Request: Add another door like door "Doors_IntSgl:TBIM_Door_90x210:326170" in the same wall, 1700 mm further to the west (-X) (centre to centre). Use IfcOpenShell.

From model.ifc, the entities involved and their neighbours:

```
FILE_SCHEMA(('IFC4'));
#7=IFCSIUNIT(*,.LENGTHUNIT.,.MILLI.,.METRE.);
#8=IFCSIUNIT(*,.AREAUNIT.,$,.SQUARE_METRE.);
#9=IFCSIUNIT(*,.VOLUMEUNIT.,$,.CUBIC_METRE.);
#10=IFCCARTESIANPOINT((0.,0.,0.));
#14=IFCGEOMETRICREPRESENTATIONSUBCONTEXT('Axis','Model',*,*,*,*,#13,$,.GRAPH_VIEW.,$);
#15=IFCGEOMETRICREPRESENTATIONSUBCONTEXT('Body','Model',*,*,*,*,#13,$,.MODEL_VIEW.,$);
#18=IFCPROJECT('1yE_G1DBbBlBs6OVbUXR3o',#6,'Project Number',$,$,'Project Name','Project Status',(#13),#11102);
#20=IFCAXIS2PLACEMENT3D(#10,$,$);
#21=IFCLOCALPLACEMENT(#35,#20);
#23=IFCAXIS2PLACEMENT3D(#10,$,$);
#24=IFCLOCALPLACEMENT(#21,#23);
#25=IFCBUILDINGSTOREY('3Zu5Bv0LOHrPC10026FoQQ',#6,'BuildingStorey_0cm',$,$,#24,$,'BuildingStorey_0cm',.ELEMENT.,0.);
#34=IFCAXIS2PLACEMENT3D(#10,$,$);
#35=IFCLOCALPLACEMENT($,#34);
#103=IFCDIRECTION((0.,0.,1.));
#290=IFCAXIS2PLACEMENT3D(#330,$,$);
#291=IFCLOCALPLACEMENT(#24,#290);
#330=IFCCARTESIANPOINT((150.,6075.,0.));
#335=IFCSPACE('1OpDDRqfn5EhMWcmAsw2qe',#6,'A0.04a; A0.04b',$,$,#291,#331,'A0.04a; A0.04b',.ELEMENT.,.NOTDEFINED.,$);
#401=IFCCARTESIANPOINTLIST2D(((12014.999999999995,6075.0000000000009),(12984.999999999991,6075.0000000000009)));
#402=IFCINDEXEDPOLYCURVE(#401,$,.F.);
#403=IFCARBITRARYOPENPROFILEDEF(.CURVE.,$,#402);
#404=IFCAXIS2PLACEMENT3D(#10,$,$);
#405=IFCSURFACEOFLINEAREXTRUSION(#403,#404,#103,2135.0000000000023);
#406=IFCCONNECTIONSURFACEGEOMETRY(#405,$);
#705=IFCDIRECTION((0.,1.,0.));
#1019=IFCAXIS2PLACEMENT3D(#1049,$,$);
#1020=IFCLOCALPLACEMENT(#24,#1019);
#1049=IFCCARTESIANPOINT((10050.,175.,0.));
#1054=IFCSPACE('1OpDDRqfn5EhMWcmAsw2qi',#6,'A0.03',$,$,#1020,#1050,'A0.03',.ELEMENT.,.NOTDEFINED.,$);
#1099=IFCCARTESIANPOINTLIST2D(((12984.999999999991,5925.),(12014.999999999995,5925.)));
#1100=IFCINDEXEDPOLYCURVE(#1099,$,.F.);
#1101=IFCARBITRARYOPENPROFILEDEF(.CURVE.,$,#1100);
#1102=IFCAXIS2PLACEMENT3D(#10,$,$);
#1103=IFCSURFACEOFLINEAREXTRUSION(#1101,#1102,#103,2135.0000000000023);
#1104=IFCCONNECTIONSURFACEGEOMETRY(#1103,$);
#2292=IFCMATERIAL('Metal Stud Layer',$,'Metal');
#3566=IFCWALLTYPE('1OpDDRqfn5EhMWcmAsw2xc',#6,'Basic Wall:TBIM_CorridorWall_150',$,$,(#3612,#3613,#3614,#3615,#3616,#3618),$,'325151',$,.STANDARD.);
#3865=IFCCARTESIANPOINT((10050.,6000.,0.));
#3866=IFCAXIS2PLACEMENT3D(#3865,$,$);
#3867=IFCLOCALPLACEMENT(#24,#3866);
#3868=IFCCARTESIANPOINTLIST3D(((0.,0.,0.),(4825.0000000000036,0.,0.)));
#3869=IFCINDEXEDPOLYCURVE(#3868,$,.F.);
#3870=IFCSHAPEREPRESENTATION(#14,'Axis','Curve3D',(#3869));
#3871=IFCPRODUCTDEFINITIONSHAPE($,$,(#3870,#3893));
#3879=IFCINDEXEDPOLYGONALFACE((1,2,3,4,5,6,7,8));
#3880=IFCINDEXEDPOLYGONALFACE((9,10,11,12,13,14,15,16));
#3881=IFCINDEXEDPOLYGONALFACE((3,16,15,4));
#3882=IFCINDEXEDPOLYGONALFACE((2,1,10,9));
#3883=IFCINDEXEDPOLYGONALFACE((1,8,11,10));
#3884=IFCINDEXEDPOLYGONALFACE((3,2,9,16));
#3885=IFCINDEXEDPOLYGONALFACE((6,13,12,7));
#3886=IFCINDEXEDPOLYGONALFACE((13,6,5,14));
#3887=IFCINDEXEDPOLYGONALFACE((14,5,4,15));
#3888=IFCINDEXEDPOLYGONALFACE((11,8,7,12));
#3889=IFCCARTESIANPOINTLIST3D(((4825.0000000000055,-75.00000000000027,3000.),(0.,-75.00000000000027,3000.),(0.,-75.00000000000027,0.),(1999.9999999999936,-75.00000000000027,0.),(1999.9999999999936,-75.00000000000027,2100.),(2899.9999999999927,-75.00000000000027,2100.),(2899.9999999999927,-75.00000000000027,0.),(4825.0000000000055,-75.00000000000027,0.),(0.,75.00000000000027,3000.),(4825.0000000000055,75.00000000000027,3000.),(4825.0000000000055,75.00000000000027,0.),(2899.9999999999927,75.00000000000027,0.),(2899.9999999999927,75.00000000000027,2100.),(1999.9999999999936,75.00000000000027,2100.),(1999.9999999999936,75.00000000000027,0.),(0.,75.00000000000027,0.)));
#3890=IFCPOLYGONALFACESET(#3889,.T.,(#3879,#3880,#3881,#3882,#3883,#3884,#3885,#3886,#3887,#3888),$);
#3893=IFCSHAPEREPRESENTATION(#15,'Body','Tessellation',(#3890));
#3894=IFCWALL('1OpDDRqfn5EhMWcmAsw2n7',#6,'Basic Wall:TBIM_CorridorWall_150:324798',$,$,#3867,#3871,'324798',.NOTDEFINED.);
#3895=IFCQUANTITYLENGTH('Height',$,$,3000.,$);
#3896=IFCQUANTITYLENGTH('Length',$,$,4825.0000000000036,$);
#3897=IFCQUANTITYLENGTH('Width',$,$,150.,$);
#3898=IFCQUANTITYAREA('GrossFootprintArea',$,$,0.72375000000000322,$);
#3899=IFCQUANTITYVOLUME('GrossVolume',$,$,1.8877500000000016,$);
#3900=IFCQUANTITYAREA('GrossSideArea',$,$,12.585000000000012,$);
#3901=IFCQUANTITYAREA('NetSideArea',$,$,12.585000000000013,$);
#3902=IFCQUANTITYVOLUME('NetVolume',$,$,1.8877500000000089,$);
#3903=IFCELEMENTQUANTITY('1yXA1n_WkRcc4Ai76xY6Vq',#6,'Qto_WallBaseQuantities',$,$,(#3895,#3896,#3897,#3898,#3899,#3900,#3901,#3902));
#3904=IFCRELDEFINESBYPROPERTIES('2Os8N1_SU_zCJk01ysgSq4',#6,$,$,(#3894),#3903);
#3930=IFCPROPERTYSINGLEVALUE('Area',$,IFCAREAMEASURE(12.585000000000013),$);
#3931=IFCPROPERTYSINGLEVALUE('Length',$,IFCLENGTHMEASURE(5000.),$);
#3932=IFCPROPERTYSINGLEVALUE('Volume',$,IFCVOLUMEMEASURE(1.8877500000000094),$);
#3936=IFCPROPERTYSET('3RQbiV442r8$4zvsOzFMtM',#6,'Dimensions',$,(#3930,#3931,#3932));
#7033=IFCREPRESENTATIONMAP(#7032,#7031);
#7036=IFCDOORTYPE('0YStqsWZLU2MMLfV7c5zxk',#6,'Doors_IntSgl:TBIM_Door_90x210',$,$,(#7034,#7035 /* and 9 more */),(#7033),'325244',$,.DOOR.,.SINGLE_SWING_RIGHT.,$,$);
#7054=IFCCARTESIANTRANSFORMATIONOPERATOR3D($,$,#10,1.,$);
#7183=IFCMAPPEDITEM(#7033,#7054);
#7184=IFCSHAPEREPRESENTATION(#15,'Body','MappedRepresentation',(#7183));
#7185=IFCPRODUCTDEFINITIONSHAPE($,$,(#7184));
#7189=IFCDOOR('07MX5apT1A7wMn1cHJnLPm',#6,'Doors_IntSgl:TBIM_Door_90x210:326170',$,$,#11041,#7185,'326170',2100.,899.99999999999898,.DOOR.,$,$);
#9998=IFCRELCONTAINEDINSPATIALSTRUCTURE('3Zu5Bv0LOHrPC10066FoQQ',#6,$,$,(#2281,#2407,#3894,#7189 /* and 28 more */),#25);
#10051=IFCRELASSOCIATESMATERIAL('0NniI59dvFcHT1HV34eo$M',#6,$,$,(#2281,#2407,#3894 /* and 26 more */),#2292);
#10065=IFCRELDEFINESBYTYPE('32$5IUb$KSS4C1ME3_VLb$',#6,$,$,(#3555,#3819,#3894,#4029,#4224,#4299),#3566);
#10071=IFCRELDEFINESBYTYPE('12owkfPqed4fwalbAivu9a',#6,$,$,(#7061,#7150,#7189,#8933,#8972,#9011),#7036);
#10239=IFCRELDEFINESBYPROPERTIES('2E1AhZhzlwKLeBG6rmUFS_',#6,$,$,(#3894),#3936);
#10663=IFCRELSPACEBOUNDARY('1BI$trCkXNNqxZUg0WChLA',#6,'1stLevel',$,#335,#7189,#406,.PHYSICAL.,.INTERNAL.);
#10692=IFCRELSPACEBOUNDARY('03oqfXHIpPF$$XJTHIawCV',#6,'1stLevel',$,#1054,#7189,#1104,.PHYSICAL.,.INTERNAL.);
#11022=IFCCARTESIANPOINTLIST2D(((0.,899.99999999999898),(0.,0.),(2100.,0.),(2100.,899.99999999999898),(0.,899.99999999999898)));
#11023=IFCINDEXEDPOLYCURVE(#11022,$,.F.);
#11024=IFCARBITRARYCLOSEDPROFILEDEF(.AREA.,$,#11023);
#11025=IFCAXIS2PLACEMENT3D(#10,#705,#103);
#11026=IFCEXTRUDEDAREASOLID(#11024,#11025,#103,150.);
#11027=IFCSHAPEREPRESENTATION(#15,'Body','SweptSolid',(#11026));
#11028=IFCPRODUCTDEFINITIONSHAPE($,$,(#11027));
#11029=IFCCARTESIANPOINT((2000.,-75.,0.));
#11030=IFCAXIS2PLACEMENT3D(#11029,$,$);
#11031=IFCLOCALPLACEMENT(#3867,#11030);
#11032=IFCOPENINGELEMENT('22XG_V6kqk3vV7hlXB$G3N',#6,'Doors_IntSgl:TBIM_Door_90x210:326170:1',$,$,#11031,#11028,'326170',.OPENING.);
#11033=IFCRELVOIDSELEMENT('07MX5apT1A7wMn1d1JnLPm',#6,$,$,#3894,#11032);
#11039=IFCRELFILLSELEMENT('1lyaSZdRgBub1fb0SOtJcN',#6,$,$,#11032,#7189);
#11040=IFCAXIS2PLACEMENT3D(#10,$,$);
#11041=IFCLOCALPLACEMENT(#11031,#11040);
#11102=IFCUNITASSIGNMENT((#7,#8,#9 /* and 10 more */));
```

```python
import numpy as np
import ifcopenshell
import ifcopenshell.api.feature
import ifcopenshell.api.geometry
import ifcopenshell.api.pset
import ifcopenshell.api.root
import ifcopenshell.geom
import ifcopenshell.util.element
import ifcopenshell.util.placement
import ifcopenshell.util.shape
import ifcopenshell.util.unit

model = ifcopenshell.open("model.ifc")
unit_scale = ifcopenshell.util.unit.calculate_unit_scale(model)
area_scale = ifcopenshell.util.unit.calculate_unit_scale(model, "AREAUNIT")
volume_scale = ifcopenshell.util.unit.calculate_unit_scale(model, "VOLUMEUNIT")
settings = ifcopenshell.geom.settings()


def volume(element):
    """Net volume in cubic metres, openings subtracted."""
    shape = ifcopenshell.geom.create_shape(settings, element)
    return ifcopenshell.util.shape.get_volume(shape.geometry)


def reuse_history(source, copy):
    """copy_class also copies each property set's owner history, people and application; keep the originals."""
    for rel in copy.IsDefinedBy:
        if rel.is_a("IfcRelDefinesByProperties") and (history := rel.RelatingPropertyDefinition.OwnerHistory):
            rel.RelatingPropertyDefinition.OwnerHistory = source.OwnerHistory
            ifcopenshell.util.element.remove_deep2(model, history)


door = model.by_guid("07MX5apT1A7wMn1cHJnLPm")
opening = door.FillsVoids[0].RelatingOpeningElement
wall = opening.VoidsElements[0].RelatingBuildingElement
before = volume(wall)
shift = ifcopenshell.util.placement.get_local_placement(wall.ObjectPlacement)[:3, 0] * -1.7 / unit_scale

# copy_class copies the void relationship, type, container and properties, but no geometry.
new_opening = ifcopenshell.api.root.copy_class(model, product=opening)
new_opening.Representation = ifcopenshell.util.element.copy_deep(
    model, opening.Representation, exclude=["IfcGeometricRepresentationContext", "IfcRepresentationMap"]
)
new_opening.Name = "Doors_IntSgl:TBIM_Door_90x210"
new_opening.Tag = None
reuse_history(opening, new_opening)
new_door = ifcopenshell.api.root.copy_class(model, product=door)
new_door.Representation = ifcopenshell.util.element.copy_deep(
    model, door.Representation, exclude=["IfcGeometricRepresentationContext", "IfcRepresentationMap"]
)
new_door.Name = "Doors_IntSgl:TBIM_Door_90x210"
new_door.Tag = None
reuse_history(door, new_door)
ifcopenshell.api.feature.add_filling(model, opening=new_opening, element=new_door)

for old, new in ((opening, new_opening), (door, new_door)):
    matrix = ifcopenshell.util.placement.get_local_placement(old.ObjectPlacement)
    matrix[:3, 3] += shift
    ifcopenshell.api.geometry.edit_object_placement(model, product=new, matrix=matrix, is_si=False)

# The copied space boundaries still share their surfaces with the original.
for rel in new_door.ProvidesBoundaries:
    if rel.ConnectionGeometry:
        rel.ConnectionGeometry = ifcopenshell.util.element.copy_deep(model, rel.ConnectionGeometry)

# Space boundary surfaces are stored in each space's coordinates; move them too.
for rel in new_door.ProvidesBoundaries:
    if not rel.ConnectionGeometry:
        continue
    surface = rel.ConnectionGeometry.SurfaceOnRelatingElement
    space_matrix = ifcopenshell.util.placement.get_local_placement(rel.RelatingSpace.ObjectPlacement)
    point = np.array(surface.Position.Location.Coordinates) + space_matrix[:3, :3].T @ shift
    surface.Position = model.createIfcAxis2Placement3D(
        model.createIfcCartesianPoint(point.tolist()), surface.Position.Axis, surface.Position.RefDirection
    )

after = volume(wall)
thickness = 0.15  # wall thickness in metres

# Update the wall's stored quantities.
qto = model.by_id(ifcopenshell.util.element.get_pset(wall, "Qto_WallBaseQuantities", should_inherit=False)["id"])
ifcopenshell.api.pset.edit_qto(model, qto=qto, properties={
    "NetSideArea": after / thickness / area_scale,
    "NetVolume": after / volume_scale,
})
pset = model.by_id(ifcopenshell.util.element.get_pset(wall, "Dimensions", should_inherit=False)["id"])
ifcopenshell.api.pset.edit_pset(model, pset=pset, properties={
    "Area": model.create_entity("IfcAreaMeasure", after / thickness / area_scale),
    "Volume": model.create_entity("IfcVolumeMeasure", after / volume_scale),
})

print(f"wall volume {before:.3f} -> {after:.3f} m3")

model.write("model_updated.ifc")
```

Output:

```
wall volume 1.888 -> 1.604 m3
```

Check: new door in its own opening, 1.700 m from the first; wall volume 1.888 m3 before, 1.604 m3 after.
